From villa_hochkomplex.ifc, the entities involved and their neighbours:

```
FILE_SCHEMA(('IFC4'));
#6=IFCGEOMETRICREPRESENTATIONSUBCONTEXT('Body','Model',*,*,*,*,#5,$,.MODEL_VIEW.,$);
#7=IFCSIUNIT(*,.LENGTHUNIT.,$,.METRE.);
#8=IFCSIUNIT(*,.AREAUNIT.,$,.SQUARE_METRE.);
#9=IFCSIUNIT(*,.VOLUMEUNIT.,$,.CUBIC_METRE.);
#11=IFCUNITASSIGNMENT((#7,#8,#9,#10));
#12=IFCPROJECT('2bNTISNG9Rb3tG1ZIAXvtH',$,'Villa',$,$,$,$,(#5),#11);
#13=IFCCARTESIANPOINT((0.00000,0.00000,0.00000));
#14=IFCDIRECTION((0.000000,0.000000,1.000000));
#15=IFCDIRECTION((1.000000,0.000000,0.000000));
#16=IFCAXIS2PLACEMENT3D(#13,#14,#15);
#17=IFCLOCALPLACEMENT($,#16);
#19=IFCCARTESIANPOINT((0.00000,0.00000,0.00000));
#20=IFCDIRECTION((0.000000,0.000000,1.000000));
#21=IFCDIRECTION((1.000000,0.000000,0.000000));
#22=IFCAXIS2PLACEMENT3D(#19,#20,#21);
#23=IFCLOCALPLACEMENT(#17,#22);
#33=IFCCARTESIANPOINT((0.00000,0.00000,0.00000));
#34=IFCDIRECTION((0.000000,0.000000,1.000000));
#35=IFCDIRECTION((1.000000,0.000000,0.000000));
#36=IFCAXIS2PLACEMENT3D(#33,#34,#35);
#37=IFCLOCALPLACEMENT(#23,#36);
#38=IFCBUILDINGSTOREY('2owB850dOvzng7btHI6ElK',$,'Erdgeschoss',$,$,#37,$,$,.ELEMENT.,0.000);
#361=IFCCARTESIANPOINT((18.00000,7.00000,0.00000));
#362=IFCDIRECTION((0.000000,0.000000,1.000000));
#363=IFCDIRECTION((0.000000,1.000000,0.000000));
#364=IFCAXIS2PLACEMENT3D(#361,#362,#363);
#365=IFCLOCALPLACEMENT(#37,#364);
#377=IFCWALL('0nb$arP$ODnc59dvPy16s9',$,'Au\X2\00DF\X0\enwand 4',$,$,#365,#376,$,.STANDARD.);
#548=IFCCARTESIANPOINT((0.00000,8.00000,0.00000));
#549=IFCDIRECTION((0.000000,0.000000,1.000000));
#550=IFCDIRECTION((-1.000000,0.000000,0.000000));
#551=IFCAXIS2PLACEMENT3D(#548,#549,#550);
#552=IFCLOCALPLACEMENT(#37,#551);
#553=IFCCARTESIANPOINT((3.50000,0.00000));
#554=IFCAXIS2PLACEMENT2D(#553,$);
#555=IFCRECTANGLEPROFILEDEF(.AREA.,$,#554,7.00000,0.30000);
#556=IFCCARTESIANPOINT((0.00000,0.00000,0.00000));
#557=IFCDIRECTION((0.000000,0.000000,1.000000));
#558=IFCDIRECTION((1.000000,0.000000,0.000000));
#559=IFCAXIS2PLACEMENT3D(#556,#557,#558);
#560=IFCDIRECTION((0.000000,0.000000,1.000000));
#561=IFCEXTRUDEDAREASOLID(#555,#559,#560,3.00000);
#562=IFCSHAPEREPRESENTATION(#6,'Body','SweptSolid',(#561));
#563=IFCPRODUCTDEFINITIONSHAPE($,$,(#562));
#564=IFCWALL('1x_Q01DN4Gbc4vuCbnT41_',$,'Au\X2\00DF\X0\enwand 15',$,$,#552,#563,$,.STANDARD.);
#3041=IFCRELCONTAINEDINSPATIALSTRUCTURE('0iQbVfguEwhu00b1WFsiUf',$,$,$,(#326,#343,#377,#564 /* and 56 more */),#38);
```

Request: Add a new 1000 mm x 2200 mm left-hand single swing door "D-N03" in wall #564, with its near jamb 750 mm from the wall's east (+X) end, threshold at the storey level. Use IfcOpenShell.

```python
import numpy as np
import ifcopenshell
import ifcopenshell.api.feature
import ifcopenshell.api.geometry
import ifcopenshell.api.root
import ifcopenshell.api.spatial
import ifcopenshell.geom
import ifcopenshell.util.element
import ifcopenshell.util.placement
import ifcopenshell.util.representation
import ifcopenshell.util.shape
import ifcopenshell.util.unit

model = ifcopenshell.open("villa_hochkomplex.ifc")
unit_scale = ifcopenshell.util.unit.calculate_unit_scale(model)
settings = ifcopenshell.geom.settings()


def volume(element):
    """Net volume in cubic metres, openings subtracted."""
    shape = ifcopenshell.geom.create_shape(settings, element)
    return ifcopenshell.util.shape.get_volume(shape.geometry)


wall = model.by_guid("1x_Q01DN4Gbc4vuCbnT41_")
storey = ifcopenshell.util.element.get_container(wall, ifc_class="IfcBuildingStorey")
context = ifcopenshell.util.representation.get_context(model, "Model", "Body", "MODEL_VIEW")
before = volume(wall)

width, height, from_end, sill = 1, 2.2, 0.75, 0.0  # metres

# The wall runs along its own X axis, and the end named is its -X end.
wall_shape = ifcopenshell.geom.create_shape(settings, wall)
x, y, z = ifcopenshell.util.shape.get_vertices(wall_shape.geometry).T
start = x.min() + from_end
face, thickness = float(y.min()), float(y.max() - y.min())
wall_matrix = ifcopenshell.util.placement.get_local_placement(wall.ObjectPlacement)
level = ifcopenshell.util.placement.get_local_placement(storey.ObjectPlacement)[2, 3]


def in_wall(x, y):
    """Placement at x, y metres in the wall's axes, at sill height."""
    matrix = wall_matrix.copy()
    matrix[:, 3] = wall_matrix @ np.array([x / unit_scale, y / unit_scale, 0.0, 1.0])
    matrix[2, 3] = level + sill / unit_scale
    return matrix


# Opening: a box that overshoots both wall faces by 50 mm.
opening = ifcopenshell.api.root.create_entity(model, ifc_class="IfcOpeningElement", predefined_type="OPENING")
box = ifcopenshell.api.geometry.add_wall_representation(
    model, context=context, length=width, height=height, thickness=thickness + 0.1
)
ifcopenshell.api.geometry.assign_representation(model, product=opening, representation=box)
ifcopenshell.api.geometry.edit_object_placement(model, product=opening, matrix=in_wall(start, face - 0.05), is_si=False)
ifcopenshell.api.feature.add_feature(model, feature=opening, element=wall)

door = ifcopenshell.api.root.create_entity(model, ifc_class="IfcDoor", name="D-N03", predefined_type="DOOR")
door.OverallWidth, door.OverallHeight = width / unit_scale, height / unit_scale
door.OperationType = "SINGLE_SWING_LEFT"
body = ifcopenshell.api.geometry.add_door_representation(
    model,
    context=context,
    overall_width=door.OverallWidth,
    overall_height=door.OverallHeight,
    operation_type="SINGLE_SWING_LEFT",
    lining_properties={"LiningDepth": thickness / unit_scale, "ThresholdDepth": thickness / unit_scale},
)
ifcopenshell.api.geometry.assign_representation(model, product=door, representation=body)
ifcopenshell.api.spatial.assign_container(model, products=[door], relating_structure=storey)
ifcopenshell.api.feature.add_filling(model, opening=opening, element=door)

# The lining spans the wall, so the door starts at the wall face.
ifcopenshell.api.geometry.edit_object_placement(model, product=door, matrix=in_wall(start, face), is_si=False)

after = volume(wall)

print(f"wall volume {before:.3f} -> {after:.3f} m3")

model.write("villa_hochkomplex_edited.ifc")
```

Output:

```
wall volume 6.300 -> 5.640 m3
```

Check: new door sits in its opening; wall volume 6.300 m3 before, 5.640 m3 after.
